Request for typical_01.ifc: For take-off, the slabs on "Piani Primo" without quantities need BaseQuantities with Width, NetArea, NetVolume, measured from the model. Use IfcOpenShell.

First a look at what the model holds.

```python
import ifcopenshell
import ifcopenshell.util.element
import ifcopenshell.util.unit

model = ifcopenshell.open("typical_01.ifc")
print(model.schema)
for unit_type in ("LENGTHUNIT", "AREAUNIT", "VOLUMEUNIT"):
    print(unit_type, ifcopenshell.util.unit.calculate_unit_scale(model, unit_type))
storey = next(s for s in model.by_type("IfcBuildingStorey") if s.Name == "Piani Primo")
slabs = [e for e in ifcopenshell.util.element.get_decomposition(storey) if e.is_a("IfcSlab")]
for e in sorted(slabs, key=lambda e: e.id()):
    print(e.id(), e.is_a(), e.Name, list(ifcopenshell.util.element.get_psets(e, qtos_only=True)), sep=" | ")
```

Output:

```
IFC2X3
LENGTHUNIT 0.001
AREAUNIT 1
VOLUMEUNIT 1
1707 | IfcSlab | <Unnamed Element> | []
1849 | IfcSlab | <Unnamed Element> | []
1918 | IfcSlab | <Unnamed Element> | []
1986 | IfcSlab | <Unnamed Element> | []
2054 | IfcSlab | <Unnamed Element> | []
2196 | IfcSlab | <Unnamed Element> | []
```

```python
import ifcopenshell
import ifcopenshell.api.pset
import ifcopenshell.geom
import ifcopenshell.util.element
import ifcopenshell.util.shape
import ifcopenshell.util.unit

model = ifcopenshell.open("typical_01.ifc")
unit_scale = ifcopenshell.util.unit.calculate_unit_scale(model)
area_scale = ifcopenshell.util.unit.calculate_unit_scale(model, "AREAUNIT")
volume_scale = ifcopenshell.util.unit.calculate_unit_scale(model, "VOLUMEUNIT")
settings = ifcopenshell.geom.settings()

storey = next(s for s in model.by_type("IfcBuildingStorey") if s.Name == "Piani Primo")
slabs = [e for e in ifcopenshell.util.element.get_decomposition(storey) if e.is_a("IfcSlab")]

for e in sorted(slabs, key=lambda e: e.id()):
    if ifcopenshell.util.element.get_psets(e, qtos_only=True, should_inherit=False):
        continue
    # Geometry comes back in metres, in the element's own axes.
    shape = ifcopenshell.geom.create_shape(settings, e)
    values = {
        "Width": ifcopenshell.util.shape.get_z(shape.geometry) / unit_scale,
        "NetArea": ifcopenshell.util.shape.get_footprint_area(shape.geometry) / area_scale,
        "NetVolume": ifcopenshell.util.shape.get_volume(shape.geometry) / volume_scale,
    }
    qto = ifcopenshell.api.pset.add_qto(model, product=e, name="BaseQuantities")
    ifcopenshell.api.pset.edit_qto(model, qto=qto, properties=values)
    print(e.id(), {k: round(v, 3) for k, v in values.items()})

model.write("typical_01_edited.ifc")
```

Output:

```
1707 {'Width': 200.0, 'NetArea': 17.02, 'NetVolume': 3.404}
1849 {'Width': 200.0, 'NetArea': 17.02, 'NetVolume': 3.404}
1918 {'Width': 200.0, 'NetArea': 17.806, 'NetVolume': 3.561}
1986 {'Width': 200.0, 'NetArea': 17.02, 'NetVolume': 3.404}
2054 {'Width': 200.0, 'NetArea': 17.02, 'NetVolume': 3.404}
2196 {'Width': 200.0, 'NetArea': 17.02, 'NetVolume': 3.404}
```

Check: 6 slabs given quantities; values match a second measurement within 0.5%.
